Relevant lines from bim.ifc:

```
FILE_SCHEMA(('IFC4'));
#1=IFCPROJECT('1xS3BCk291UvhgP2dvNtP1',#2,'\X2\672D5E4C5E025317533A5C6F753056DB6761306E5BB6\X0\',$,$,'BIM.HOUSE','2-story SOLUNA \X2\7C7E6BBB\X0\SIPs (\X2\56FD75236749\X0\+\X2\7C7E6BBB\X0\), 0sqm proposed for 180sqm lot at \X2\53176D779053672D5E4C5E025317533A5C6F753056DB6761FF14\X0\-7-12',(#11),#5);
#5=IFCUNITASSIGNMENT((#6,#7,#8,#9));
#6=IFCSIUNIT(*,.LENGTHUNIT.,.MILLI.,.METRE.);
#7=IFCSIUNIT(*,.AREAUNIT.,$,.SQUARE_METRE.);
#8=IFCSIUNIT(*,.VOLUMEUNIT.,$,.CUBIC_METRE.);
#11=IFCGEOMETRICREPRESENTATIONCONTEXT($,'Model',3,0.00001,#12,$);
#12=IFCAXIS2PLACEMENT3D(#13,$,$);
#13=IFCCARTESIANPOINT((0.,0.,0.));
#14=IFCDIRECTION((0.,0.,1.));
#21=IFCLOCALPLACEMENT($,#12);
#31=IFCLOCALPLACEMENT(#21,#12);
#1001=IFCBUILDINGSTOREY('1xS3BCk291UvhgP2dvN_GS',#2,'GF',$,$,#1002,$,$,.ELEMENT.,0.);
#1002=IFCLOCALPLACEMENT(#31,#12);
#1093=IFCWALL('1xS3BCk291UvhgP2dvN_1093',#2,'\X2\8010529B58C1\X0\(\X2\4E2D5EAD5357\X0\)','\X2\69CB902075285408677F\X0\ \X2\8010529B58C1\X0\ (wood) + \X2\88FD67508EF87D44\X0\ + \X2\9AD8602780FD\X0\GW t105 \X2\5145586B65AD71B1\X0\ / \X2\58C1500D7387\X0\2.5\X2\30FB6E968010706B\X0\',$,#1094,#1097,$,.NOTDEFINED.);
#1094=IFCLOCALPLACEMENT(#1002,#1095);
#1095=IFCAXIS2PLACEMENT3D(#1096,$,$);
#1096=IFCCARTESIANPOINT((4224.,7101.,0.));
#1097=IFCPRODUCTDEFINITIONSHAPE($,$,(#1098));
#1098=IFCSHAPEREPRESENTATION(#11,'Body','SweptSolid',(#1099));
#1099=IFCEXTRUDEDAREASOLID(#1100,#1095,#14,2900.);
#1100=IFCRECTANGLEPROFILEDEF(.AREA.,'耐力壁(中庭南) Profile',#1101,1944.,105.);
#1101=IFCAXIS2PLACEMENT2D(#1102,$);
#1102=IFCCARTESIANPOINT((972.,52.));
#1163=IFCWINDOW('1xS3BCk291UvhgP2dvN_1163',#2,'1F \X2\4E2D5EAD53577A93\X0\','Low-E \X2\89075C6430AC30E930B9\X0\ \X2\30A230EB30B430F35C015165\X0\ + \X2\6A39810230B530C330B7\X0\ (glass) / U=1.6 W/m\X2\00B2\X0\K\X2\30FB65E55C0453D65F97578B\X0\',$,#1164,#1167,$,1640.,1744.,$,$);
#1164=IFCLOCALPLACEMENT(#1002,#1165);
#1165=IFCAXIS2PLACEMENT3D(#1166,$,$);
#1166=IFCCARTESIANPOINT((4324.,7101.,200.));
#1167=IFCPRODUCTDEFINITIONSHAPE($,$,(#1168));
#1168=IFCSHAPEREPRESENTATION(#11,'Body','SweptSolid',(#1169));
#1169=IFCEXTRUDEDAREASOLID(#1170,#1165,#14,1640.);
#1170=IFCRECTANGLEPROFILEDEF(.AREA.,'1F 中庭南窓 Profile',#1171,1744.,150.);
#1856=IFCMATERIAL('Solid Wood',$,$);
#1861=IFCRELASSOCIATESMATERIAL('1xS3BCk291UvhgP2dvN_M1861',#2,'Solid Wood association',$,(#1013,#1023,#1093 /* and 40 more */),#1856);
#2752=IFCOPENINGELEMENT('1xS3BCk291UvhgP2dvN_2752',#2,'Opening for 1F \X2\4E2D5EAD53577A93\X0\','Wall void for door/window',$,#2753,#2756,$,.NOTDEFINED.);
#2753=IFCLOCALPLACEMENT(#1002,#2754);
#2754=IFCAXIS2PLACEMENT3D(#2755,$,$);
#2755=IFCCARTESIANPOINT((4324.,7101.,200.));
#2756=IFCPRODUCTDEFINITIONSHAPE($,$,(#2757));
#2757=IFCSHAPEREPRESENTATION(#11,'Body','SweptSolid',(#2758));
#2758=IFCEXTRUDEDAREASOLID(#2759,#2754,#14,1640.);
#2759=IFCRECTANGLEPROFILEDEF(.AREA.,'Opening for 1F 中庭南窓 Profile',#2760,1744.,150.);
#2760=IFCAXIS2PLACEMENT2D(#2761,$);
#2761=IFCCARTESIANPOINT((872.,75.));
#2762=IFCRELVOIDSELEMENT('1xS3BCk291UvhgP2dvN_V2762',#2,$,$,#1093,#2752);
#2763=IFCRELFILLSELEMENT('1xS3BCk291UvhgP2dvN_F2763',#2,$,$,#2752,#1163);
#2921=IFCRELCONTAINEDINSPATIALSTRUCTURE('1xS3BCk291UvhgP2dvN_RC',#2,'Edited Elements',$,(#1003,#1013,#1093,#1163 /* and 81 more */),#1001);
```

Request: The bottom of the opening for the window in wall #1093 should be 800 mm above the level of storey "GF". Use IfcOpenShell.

```python
import numpy as np
import ifcopenshell
import ifcopenshell.api.geometry
import ifcopenshell.geom
import ifcopenshell.util.element
import ifcopenshell.util.placement
import ifcopenshell.util.shape
import ifcopenshell.util.unit

model = ifcopenshell.open("bim.ifc")
unit_scale = ifcopenshell.util.unit.calculate_unit_scale(model)

window = model.by_guid("1xS3BCk291UvhgP2dvN_1163")
opening = window.FillsVoids[0].RelatingOpeningElement
storey = ifcopenshell.util.element.get_container(window, ifc_class="IfcBuildingStorey")
level = ifcopenshell.util.placement.get_local_placement(storey.ObjectPlacement)[2, 3]

# The opening's origin need not be at the sill, so measure its lowest point.
shape = ifcopenshell.geom.create_shape(ifcopenshell.geom.settings(), opening)
bottom = ifcopenshell.util.shape.get_shape_bottom_elevation(shape, shape.geometry) / unit_scale
dz = level + 0.8 / unit_scale - bottom

shift = np.array([0.0, 0.0, dz])
# The window is not placed relative to its opening, so move both.
for product in (opening, window):
    matrix = ifcopenshell.util.placement.get_local_placement(product.ObjectPlacement)
    matrix[:3, 3] += shift
    ifcopenshell.api.geometry.edit_object_placement(model, product=product, matrix=matrix, is_si=False)

print(f"moved by {dz * unit_scale:+.3f} m")

model.write("bim_updated.ifc")
```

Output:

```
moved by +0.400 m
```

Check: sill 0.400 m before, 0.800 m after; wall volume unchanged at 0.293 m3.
